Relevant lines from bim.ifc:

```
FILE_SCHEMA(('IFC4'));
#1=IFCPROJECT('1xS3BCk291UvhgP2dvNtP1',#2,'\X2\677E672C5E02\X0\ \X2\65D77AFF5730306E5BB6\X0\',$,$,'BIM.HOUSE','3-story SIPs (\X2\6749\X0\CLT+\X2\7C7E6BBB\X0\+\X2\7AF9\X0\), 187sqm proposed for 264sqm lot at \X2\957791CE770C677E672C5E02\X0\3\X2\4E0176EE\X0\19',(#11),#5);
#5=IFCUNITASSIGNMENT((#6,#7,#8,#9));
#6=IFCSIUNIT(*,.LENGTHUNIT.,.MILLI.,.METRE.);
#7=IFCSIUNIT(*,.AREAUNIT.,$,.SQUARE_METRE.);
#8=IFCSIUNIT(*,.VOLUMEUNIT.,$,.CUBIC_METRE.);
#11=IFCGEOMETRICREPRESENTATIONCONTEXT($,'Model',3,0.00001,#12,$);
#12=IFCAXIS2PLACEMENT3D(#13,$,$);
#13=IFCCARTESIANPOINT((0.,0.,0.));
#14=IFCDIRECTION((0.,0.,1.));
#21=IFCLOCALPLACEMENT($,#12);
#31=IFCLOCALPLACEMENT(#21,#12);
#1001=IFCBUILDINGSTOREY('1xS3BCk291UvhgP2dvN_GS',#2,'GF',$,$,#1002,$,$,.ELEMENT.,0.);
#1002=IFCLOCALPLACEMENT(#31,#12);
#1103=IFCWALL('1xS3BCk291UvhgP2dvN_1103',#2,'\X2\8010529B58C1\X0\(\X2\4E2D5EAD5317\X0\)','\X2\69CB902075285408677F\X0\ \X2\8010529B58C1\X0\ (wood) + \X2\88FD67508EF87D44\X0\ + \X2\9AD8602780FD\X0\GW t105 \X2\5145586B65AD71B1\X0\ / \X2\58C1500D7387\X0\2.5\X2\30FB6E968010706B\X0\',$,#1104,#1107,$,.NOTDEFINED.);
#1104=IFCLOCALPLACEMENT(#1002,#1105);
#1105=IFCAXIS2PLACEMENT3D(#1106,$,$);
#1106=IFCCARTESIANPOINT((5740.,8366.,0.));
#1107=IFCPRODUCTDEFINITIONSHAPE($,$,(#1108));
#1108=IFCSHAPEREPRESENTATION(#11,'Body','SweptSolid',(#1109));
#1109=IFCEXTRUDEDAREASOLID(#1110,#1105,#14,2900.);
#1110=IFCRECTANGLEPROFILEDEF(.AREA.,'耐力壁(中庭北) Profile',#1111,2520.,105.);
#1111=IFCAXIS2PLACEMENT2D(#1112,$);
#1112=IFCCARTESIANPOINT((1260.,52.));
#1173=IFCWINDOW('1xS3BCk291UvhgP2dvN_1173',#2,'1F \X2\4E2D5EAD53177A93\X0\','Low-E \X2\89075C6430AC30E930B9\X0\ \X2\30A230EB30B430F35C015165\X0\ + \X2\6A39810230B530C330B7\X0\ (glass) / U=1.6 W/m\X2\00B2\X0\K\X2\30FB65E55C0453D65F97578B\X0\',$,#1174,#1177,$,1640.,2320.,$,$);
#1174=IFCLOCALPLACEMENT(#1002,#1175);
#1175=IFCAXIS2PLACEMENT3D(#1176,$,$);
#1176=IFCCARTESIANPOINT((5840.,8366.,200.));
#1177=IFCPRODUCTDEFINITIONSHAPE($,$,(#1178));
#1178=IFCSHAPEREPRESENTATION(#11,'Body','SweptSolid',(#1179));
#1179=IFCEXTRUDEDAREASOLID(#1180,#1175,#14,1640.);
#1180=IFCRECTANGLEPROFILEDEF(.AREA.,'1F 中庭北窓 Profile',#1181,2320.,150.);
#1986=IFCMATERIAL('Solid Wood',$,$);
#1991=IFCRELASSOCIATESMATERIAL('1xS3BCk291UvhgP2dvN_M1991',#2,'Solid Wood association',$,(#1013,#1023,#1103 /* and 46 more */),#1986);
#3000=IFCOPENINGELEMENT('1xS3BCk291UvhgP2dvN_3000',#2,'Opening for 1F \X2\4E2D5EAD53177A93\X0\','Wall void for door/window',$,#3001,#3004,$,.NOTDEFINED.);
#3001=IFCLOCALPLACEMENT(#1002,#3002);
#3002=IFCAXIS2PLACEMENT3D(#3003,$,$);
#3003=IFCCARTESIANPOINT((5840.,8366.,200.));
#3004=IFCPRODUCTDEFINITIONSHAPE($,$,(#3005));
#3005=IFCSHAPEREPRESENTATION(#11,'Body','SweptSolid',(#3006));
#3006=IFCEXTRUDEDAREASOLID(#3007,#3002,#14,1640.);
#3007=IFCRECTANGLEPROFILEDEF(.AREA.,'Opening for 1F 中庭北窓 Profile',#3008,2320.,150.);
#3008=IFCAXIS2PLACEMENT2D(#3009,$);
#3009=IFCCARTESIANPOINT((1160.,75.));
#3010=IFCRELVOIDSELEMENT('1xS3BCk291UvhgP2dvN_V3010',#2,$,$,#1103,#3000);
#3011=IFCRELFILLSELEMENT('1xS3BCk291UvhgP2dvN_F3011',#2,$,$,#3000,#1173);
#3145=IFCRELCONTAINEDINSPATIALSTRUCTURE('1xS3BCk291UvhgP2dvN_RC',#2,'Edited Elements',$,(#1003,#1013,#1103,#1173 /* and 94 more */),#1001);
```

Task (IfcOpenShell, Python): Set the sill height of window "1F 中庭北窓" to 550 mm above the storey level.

```python
import numpy as np
import ifcopenshell
import ifcopenshell.api.geometry
import ifcopenshell.geom
import ifcopenshell.util.element
import ifcopenshell.util.placement
import ifcopenshell.util.shape
import ifcopenshell.util.unit

model = ifcopenshell.open("bim.ifc")
unit_scale = ifcopenshell.util.unit.calculate_unit_scale(model)

window = model.by_id(1173)
opening = window.FillsVoids[0].RelatingOpeningElement
storey = ifcopenshell.util.element.get_container(window, ifc_class="IfcBuildingStorey")
level = ifcopenshell.util.placement.get_local_placement(storey.ObjectPlacement)[2, 3]

# The opening's origin need not be at the sill, so measure its lowest point.
shape = ifcopenshell.geom.create_shape(ifcopenshell.geom.settings(), opening)
bottom = ifcopenshell.util.shape.get_shape_bottom_elevation(shape, shape.geometry) / unit_scale
dz = level + 550.0 - bottom

shift = np.array([0.0, 0.0, dz])
# The window is not placed relative to its opening, so move both.
for product in (opening, window):
    matrix = ifcopenshell.util.placement.get_local_placement(product.ObjectPlacement)
    matrix[:3, 3] += shift
    ifcopenshell.api.geometry.edit_object_placement(model, product=product, matrix=matrix, is_si=False)

print(f"moved by {dz * unit_scale:+.3f} m")

model.write("bim-out.ifc")
```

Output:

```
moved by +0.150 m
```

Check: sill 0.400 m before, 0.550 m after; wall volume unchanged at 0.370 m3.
